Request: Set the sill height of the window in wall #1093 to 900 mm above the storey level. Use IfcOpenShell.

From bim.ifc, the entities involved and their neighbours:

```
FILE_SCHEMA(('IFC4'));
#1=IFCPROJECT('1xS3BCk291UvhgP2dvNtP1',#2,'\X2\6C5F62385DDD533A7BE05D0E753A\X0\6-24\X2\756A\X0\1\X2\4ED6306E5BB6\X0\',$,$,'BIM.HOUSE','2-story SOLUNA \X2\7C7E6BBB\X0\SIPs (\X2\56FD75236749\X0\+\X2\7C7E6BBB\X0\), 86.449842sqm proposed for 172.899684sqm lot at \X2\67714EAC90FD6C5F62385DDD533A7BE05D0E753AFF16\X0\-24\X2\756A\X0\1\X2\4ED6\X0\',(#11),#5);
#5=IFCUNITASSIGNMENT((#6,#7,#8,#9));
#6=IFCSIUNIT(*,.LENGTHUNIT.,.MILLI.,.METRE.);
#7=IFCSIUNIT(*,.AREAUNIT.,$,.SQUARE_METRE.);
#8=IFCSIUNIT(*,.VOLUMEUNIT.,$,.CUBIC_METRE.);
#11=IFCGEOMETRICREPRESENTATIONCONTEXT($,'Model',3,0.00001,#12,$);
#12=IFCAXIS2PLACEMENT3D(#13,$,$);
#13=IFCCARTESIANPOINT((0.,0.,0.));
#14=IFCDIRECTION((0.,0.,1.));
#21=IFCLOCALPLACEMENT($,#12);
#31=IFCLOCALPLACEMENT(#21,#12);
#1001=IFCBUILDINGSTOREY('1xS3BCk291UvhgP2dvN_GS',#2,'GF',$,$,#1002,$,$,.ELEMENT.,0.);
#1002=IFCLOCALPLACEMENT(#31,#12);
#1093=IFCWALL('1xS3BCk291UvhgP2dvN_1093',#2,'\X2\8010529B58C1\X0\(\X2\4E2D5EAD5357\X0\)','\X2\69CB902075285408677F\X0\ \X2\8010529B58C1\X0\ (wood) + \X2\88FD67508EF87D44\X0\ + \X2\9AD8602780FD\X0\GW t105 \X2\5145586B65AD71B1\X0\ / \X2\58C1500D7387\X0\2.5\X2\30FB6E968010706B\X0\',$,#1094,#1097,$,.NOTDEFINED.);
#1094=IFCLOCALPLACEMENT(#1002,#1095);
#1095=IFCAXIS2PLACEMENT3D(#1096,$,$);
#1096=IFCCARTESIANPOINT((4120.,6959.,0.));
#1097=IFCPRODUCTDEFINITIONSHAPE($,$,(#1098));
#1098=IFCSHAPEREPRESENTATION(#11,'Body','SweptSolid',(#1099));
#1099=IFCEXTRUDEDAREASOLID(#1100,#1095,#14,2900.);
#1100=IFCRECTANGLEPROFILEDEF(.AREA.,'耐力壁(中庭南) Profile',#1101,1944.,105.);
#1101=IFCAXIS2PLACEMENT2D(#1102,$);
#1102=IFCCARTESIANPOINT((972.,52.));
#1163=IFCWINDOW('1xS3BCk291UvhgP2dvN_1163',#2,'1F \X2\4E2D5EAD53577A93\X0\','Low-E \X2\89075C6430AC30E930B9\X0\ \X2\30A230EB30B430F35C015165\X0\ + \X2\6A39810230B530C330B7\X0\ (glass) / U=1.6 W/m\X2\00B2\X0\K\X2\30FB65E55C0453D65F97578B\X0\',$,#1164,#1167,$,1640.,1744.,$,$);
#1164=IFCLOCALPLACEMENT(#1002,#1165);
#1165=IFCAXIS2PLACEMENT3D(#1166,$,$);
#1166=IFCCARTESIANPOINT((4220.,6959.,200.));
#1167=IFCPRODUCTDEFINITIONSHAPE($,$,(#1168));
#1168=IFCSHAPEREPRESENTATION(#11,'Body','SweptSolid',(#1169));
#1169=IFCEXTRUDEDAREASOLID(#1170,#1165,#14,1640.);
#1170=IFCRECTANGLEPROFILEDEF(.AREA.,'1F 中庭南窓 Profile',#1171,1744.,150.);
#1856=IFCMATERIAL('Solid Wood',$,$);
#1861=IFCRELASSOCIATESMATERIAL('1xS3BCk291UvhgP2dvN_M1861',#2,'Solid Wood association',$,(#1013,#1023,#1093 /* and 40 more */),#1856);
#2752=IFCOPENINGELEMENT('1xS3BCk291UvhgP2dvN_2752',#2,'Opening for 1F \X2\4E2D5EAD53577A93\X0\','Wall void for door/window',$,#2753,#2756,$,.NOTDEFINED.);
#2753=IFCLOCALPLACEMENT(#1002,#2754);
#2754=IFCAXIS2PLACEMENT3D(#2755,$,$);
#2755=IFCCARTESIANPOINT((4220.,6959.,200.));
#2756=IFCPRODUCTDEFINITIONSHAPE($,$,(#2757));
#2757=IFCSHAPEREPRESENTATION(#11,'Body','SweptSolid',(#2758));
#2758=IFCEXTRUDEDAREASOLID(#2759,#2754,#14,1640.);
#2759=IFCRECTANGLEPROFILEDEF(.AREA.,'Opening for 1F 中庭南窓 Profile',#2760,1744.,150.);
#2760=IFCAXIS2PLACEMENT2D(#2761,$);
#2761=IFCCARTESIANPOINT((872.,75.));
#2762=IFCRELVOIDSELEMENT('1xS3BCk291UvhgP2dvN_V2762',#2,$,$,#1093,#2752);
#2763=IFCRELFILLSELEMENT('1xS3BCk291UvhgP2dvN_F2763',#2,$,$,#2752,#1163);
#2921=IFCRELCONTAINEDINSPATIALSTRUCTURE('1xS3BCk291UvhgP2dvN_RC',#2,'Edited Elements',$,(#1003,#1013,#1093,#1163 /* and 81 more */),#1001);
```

```python
import numpy as np
import ifcopenshell
import ifcopenshell.api.geometry
import ifcopenshell.geom
import ifcopenshell.util.element
import ifcopenshell.util.placement
import ifcopenshell.util.shape
import ifcopenshell.util.unit

model = ifcopenshell.open("bim.ifc")
unit_scale = ifcopenshell.util.unit.calculate_unit_scale(model)

window = model.by_id(1163)
opening = window.FillsVoids[0].RelatingOpeningElement
storey = ifcopenshell.util.element.get_container(window, ifc_class="IfcBuildingStorey")
level = ifcopenshell.util.placement.get_local_placement(storey.ObjectPlacement)[2, 3]

# The opening's origin need not be at the sill, so measure its lowest point.
shape = ifcopenshell.geom.create_shape(ifcopenshell.geom.settings(), opening)
bottom = ifcopenshell.util.shape.get_shape_bottom_elevation(shape, shape.geometry) / unit_scale
dz = level + 0.9 / unit_scale - bottom

shift = np.array([0.0, 0.0, dz])
# The window is not placed relative to its opening, so move both.
for product in (opening, window):
    matrix = ifcopenshell.util.placement.get_local_placement(product.ObjectPlacement)
    matrix[:3, 3] += shift
    ifcopenshell.api.geometry.edit_object_placement(model, product=product, matrix=matrix, is_si=False)

print(f"moved by {dz * unit_scale:+.3f} m")

model.write("bim_rev.ifc")
```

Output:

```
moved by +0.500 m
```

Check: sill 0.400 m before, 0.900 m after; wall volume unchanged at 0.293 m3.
